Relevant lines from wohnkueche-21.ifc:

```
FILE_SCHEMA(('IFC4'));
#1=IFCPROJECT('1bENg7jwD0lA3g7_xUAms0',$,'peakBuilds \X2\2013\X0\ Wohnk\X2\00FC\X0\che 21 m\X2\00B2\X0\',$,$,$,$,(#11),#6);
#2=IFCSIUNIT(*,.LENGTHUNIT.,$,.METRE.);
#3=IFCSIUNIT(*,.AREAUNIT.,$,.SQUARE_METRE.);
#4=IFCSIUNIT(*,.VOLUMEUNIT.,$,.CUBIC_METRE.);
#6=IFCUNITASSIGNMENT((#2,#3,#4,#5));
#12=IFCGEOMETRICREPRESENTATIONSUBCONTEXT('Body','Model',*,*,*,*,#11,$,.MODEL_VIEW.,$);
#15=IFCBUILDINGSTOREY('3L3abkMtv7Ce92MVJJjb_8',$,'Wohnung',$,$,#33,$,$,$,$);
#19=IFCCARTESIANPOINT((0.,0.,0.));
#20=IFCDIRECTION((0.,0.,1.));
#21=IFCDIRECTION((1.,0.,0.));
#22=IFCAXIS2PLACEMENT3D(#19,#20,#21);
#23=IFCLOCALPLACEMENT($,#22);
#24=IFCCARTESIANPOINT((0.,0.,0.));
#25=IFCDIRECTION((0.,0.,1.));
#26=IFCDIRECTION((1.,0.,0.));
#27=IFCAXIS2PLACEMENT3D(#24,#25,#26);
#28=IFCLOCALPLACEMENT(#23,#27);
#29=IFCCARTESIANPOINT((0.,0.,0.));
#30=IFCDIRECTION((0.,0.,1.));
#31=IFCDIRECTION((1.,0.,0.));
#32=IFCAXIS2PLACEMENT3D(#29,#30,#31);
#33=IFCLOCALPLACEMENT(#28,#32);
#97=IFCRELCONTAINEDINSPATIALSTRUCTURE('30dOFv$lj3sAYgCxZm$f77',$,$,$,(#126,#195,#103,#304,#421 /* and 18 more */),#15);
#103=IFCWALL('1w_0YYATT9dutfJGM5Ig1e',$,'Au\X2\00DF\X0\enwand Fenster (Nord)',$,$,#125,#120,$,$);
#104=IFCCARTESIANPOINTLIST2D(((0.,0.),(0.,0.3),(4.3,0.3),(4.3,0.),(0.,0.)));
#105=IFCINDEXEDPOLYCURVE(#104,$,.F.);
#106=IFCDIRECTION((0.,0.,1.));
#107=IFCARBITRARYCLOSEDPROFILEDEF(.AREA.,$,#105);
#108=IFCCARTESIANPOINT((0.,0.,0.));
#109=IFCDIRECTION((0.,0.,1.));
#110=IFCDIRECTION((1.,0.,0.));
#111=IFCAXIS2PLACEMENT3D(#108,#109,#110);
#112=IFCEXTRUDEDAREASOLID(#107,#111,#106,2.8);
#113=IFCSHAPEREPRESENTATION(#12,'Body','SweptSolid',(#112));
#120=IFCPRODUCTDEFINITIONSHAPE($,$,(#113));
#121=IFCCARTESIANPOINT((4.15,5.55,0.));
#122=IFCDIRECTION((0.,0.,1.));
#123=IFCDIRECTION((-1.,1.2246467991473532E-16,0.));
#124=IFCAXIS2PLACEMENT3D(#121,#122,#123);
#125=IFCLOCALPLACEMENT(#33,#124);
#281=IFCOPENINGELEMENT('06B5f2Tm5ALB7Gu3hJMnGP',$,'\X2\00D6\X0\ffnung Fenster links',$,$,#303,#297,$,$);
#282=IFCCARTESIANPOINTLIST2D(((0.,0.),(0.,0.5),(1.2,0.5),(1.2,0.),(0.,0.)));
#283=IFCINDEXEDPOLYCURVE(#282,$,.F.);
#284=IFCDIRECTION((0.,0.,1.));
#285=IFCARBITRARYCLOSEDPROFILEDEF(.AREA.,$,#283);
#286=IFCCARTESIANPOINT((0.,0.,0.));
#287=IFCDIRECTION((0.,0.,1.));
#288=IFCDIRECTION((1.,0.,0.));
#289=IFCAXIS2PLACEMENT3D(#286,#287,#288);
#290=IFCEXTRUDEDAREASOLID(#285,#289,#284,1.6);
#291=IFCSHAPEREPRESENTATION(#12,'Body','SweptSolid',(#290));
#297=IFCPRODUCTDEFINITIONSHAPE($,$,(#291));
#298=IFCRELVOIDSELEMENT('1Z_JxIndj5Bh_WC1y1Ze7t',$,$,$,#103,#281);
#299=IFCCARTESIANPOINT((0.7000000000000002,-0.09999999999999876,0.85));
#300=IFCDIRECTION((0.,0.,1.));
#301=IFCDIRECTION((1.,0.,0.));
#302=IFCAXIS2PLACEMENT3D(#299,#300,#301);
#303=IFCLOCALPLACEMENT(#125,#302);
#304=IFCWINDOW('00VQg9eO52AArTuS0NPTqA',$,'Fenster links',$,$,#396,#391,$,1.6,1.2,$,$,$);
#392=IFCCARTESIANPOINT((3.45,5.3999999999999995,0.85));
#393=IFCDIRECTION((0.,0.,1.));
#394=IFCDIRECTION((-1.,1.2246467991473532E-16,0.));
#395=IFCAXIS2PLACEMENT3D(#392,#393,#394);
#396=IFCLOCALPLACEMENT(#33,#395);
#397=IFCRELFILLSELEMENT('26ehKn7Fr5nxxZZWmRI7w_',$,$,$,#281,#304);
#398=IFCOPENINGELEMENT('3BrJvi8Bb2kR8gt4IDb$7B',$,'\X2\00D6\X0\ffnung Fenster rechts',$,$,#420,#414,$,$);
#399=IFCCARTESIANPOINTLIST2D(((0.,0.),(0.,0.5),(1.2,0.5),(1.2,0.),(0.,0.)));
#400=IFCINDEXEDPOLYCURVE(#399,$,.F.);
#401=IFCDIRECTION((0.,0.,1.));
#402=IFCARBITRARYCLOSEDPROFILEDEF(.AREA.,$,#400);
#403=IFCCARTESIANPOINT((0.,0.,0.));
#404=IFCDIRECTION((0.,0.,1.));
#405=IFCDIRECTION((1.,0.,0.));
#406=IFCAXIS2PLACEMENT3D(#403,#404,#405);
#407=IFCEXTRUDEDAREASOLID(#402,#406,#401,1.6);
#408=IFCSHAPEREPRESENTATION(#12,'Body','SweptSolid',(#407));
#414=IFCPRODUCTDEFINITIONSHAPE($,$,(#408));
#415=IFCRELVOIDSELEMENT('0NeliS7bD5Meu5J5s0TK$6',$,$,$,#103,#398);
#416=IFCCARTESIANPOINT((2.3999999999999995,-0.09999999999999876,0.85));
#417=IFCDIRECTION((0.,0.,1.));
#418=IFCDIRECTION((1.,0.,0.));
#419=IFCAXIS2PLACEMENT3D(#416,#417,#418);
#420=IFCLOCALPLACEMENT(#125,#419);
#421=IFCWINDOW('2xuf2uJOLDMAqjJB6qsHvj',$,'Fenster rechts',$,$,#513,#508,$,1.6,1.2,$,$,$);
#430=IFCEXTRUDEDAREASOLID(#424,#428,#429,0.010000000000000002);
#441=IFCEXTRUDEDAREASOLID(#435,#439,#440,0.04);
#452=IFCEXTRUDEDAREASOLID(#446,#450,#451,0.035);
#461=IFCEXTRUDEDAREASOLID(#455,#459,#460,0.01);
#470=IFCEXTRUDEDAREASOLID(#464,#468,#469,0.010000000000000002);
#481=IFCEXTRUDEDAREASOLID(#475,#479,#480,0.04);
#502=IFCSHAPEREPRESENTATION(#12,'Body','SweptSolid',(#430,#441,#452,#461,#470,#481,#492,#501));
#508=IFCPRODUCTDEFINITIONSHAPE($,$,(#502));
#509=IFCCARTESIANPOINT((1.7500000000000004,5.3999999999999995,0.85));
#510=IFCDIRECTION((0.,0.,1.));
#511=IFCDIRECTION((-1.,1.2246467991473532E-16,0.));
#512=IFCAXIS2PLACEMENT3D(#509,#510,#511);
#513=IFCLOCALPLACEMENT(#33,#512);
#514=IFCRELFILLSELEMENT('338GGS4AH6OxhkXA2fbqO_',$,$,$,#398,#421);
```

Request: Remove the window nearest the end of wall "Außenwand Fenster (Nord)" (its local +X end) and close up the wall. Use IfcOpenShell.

```python
import ifcopenshell
import ifcopenshell.api.feature
import ifcopenshell.api.root
import ifcopenshell.geom
import ifcopenshell.util.shape

model = ifcopenshell.open("wohnkueche-21.ifc")
settings = ifcopenshell.geom.settings()


def volume(element):
    """Net volume in cubic metres, openings subtracted."""
    shape = ifcopenshell.geom.create_shape(settings, element)
    return ifcopenshell.util.shape.get_volume(shape.geometry)


window = model.by_guid("2xuf2uJOLDMAqjJB6qsHvj")
opening = window.FillsVoids[0].RelatingOpeningElement
wall = opening.VoidsElements[0].RelatingBuildingElement
before = volume(wall)

ifcopenshell.api.root.remove_product(model, product=window)
ifcopenshell.api.feature.remove_feature(model, feature=opening)

after = volume(wall)

print(f"wall volume {before:.3f} -> {after:.3f} m3")

model.write("wohnkueche-21_updated.ifc")
```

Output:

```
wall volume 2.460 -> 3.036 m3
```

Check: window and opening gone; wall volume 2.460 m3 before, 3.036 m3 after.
